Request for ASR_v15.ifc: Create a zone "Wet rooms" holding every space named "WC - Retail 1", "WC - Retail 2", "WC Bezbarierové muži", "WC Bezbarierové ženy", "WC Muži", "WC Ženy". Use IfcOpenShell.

First a look at what the model holds.

```python
import ifcopenshell

model = ifcopenshell.open("ASR_v15.ifc")
print(model.schema)
seen = {}
for space in model.by_type("IfcSpace"):
    seen[space.LongName] = seen.get(space.LongName, 0) + 1
for name, count in sorted(seen.items(), key=str):
    print(count, "x", name)
print("zones:", [z.Name for z in model.by_type("IfcZone")][:20])
```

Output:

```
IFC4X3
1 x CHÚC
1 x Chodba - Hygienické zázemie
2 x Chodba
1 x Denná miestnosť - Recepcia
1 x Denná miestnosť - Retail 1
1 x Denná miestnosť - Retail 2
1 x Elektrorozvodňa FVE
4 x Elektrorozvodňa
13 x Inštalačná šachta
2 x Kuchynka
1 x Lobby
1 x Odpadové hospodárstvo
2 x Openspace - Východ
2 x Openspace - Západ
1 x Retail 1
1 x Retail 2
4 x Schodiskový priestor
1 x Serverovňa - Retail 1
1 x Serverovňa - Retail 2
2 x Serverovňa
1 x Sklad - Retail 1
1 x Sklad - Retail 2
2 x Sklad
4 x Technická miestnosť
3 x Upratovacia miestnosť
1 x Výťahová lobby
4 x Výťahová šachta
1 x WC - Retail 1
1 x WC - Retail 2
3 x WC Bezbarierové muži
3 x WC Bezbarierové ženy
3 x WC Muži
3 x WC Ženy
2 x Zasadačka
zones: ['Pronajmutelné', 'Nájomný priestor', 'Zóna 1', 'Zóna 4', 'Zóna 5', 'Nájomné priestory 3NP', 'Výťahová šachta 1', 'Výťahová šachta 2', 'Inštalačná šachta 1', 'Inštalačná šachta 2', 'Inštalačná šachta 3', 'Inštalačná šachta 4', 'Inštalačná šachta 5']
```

```python
import ifcopenshell
import ifcopenshell.api.group
import ifcopenshell.api.root

model = ifcopenshell.open("ASR_v15.ifc")

names = {"WC - Retail 1", "WC - Retail 2", "WC Bezbarierové muži", "WC Bezbarierové ženy", "WC Muži", "WC Ženy"}
spaces = [s for s in model.by_type("IfcSpace") if s.LongName in names]

zone = ifcopenshell.api.root.create_entity(model, ifc_class="IfcZone", name="Wet rooms")
ifcopenshell.api.group.assign_group(model, products=spaces, group=zone)
print(len(spaces), "spaces in", zone.Name)

model.write("ASR_v15_edited.ifc")
```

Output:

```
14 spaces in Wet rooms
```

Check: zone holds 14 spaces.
